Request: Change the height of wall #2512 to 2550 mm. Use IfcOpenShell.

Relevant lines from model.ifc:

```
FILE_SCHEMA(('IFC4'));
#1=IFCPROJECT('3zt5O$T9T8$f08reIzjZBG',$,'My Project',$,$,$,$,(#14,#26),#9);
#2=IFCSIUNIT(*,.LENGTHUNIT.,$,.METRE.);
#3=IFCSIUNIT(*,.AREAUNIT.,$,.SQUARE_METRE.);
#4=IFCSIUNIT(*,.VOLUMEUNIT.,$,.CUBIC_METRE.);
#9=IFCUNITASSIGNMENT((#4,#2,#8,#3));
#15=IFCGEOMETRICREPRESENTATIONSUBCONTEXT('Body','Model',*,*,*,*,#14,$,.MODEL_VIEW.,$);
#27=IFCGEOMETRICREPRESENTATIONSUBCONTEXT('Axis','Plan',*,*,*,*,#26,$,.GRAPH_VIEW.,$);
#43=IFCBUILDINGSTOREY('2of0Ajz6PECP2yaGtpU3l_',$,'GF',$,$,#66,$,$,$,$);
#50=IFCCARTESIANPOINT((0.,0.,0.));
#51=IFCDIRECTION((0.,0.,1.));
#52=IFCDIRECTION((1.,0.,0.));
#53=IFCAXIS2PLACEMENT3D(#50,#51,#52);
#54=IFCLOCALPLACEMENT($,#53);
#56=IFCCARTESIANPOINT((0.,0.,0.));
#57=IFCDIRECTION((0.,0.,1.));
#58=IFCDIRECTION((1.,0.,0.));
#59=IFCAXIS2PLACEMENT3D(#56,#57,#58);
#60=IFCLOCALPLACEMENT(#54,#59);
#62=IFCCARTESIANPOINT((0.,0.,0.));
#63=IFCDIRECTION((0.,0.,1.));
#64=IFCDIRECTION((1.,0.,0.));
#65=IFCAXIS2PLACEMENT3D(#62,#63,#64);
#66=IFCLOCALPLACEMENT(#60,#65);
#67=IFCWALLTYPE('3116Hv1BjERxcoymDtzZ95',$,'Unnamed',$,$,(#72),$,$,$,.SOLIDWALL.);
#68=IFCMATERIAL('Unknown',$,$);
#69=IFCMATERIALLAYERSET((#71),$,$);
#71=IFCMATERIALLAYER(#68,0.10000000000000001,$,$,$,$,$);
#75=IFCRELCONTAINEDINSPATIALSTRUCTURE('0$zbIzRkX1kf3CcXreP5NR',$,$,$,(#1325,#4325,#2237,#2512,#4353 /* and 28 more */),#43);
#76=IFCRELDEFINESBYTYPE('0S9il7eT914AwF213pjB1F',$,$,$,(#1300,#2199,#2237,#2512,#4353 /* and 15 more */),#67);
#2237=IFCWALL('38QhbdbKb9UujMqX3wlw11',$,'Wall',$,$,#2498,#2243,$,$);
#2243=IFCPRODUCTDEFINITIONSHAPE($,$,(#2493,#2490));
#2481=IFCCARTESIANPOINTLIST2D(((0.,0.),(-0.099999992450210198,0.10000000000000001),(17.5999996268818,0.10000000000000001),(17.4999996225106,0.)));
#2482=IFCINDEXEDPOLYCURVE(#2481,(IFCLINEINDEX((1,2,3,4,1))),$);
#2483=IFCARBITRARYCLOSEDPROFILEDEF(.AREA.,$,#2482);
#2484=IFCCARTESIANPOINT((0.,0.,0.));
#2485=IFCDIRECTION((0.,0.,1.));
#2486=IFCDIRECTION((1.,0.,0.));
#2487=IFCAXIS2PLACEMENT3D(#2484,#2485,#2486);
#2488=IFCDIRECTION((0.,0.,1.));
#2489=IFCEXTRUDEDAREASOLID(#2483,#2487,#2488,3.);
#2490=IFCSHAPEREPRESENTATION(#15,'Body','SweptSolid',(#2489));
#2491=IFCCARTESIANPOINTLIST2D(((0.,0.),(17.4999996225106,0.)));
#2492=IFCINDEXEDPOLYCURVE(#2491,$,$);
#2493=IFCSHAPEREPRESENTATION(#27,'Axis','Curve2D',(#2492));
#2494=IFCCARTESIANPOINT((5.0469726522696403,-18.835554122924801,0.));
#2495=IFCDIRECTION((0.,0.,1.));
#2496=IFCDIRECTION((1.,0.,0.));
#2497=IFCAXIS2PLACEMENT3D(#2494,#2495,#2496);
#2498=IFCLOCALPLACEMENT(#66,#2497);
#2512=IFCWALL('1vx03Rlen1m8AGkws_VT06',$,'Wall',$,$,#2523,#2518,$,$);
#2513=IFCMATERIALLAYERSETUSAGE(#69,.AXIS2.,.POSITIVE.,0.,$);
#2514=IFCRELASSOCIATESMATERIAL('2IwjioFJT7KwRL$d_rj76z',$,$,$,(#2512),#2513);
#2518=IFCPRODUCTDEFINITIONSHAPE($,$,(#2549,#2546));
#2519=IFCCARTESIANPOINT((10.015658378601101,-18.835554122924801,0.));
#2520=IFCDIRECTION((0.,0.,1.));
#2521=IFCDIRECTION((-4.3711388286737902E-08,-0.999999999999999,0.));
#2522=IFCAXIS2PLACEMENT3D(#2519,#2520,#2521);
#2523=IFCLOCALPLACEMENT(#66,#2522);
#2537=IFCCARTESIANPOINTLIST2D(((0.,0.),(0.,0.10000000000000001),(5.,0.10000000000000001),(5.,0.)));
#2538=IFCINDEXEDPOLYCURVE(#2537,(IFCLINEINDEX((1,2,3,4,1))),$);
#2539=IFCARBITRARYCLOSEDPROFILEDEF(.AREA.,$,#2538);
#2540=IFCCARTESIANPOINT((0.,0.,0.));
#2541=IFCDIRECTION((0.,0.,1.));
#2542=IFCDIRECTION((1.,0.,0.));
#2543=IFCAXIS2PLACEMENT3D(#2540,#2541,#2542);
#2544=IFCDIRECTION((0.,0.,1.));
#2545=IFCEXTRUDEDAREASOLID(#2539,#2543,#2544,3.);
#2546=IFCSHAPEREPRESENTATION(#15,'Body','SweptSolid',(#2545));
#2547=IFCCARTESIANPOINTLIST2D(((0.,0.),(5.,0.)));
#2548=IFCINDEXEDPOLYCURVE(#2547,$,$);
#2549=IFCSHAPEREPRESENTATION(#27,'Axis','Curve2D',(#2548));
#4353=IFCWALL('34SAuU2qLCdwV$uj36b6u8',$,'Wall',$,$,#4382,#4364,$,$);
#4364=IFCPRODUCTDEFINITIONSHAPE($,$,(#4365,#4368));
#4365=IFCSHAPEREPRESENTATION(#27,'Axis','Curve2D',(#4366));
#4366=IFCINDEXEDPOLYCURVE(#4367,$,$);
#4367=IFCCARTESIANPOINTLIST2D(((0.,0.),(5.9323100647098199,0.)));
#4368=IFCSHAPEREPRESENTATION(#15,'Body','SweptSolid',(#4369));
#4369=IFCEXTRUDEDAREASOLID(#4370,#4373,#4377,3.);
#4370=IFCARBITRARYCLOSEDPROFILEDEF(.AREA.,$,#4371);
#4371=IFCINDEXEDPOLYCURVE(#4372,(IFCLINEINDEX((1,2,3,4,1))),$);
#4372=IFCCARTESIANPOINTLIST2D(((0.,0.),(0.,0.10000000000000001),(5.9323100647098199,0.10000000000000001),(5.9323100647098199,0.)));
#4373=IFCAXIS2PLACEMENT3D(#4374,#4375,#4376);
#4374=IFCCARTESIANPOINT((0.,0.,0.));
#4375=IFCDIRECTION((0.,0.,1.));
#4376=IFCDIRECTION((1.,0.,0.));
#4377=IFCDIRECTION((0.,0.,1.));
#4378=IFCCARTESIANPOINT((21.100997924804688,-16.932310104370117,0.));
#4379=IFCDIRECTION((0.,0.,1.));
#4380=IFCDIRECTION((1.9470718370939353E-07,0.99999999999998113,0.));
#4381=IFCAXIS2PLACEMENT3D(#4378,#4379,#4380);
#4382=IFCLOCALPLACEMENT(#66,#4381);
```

```python
import ifcopenshell
import ifcopenshell.geom
import ifcopenshell.util.representation
import ifcopenshell.util.shape
import ifcopenshell.util.unit

model = ifcopenshell.open("model.ifc")
unit_scale = ifcopenshell.util.unit.calculate_unit_scale(model)
settings = ifcopenshell.geom.settings()


def volume(element):
    """Net volume in cubic metres, openings subtracted."""
    shape = ifcopenshell.geom.create_shape(settings, element)
    return ifcopenshell.util.shape.get_volume(shape.geometry)


wall = model.by_guid("1vx03Rlen1m8AGkws_VT06")
before = volume(wall)

body = ifcopenshell.util.representation.get_representation(wall, "Model", "Body")
solid = body.Items[0]
old_height = solid.Depth
solid.Depth = 2.55 / unit_scale
after = volume(wall)

print(f"height {old_height:g} -> {solid.Depth:g}, volume {before:.3f} -> {after:.3f} m3")

model.write("model_v2.ifc")
```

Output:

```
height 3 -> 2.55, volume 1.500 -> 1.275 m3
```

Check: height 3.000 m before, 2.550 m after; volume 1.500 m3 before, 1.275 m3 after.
